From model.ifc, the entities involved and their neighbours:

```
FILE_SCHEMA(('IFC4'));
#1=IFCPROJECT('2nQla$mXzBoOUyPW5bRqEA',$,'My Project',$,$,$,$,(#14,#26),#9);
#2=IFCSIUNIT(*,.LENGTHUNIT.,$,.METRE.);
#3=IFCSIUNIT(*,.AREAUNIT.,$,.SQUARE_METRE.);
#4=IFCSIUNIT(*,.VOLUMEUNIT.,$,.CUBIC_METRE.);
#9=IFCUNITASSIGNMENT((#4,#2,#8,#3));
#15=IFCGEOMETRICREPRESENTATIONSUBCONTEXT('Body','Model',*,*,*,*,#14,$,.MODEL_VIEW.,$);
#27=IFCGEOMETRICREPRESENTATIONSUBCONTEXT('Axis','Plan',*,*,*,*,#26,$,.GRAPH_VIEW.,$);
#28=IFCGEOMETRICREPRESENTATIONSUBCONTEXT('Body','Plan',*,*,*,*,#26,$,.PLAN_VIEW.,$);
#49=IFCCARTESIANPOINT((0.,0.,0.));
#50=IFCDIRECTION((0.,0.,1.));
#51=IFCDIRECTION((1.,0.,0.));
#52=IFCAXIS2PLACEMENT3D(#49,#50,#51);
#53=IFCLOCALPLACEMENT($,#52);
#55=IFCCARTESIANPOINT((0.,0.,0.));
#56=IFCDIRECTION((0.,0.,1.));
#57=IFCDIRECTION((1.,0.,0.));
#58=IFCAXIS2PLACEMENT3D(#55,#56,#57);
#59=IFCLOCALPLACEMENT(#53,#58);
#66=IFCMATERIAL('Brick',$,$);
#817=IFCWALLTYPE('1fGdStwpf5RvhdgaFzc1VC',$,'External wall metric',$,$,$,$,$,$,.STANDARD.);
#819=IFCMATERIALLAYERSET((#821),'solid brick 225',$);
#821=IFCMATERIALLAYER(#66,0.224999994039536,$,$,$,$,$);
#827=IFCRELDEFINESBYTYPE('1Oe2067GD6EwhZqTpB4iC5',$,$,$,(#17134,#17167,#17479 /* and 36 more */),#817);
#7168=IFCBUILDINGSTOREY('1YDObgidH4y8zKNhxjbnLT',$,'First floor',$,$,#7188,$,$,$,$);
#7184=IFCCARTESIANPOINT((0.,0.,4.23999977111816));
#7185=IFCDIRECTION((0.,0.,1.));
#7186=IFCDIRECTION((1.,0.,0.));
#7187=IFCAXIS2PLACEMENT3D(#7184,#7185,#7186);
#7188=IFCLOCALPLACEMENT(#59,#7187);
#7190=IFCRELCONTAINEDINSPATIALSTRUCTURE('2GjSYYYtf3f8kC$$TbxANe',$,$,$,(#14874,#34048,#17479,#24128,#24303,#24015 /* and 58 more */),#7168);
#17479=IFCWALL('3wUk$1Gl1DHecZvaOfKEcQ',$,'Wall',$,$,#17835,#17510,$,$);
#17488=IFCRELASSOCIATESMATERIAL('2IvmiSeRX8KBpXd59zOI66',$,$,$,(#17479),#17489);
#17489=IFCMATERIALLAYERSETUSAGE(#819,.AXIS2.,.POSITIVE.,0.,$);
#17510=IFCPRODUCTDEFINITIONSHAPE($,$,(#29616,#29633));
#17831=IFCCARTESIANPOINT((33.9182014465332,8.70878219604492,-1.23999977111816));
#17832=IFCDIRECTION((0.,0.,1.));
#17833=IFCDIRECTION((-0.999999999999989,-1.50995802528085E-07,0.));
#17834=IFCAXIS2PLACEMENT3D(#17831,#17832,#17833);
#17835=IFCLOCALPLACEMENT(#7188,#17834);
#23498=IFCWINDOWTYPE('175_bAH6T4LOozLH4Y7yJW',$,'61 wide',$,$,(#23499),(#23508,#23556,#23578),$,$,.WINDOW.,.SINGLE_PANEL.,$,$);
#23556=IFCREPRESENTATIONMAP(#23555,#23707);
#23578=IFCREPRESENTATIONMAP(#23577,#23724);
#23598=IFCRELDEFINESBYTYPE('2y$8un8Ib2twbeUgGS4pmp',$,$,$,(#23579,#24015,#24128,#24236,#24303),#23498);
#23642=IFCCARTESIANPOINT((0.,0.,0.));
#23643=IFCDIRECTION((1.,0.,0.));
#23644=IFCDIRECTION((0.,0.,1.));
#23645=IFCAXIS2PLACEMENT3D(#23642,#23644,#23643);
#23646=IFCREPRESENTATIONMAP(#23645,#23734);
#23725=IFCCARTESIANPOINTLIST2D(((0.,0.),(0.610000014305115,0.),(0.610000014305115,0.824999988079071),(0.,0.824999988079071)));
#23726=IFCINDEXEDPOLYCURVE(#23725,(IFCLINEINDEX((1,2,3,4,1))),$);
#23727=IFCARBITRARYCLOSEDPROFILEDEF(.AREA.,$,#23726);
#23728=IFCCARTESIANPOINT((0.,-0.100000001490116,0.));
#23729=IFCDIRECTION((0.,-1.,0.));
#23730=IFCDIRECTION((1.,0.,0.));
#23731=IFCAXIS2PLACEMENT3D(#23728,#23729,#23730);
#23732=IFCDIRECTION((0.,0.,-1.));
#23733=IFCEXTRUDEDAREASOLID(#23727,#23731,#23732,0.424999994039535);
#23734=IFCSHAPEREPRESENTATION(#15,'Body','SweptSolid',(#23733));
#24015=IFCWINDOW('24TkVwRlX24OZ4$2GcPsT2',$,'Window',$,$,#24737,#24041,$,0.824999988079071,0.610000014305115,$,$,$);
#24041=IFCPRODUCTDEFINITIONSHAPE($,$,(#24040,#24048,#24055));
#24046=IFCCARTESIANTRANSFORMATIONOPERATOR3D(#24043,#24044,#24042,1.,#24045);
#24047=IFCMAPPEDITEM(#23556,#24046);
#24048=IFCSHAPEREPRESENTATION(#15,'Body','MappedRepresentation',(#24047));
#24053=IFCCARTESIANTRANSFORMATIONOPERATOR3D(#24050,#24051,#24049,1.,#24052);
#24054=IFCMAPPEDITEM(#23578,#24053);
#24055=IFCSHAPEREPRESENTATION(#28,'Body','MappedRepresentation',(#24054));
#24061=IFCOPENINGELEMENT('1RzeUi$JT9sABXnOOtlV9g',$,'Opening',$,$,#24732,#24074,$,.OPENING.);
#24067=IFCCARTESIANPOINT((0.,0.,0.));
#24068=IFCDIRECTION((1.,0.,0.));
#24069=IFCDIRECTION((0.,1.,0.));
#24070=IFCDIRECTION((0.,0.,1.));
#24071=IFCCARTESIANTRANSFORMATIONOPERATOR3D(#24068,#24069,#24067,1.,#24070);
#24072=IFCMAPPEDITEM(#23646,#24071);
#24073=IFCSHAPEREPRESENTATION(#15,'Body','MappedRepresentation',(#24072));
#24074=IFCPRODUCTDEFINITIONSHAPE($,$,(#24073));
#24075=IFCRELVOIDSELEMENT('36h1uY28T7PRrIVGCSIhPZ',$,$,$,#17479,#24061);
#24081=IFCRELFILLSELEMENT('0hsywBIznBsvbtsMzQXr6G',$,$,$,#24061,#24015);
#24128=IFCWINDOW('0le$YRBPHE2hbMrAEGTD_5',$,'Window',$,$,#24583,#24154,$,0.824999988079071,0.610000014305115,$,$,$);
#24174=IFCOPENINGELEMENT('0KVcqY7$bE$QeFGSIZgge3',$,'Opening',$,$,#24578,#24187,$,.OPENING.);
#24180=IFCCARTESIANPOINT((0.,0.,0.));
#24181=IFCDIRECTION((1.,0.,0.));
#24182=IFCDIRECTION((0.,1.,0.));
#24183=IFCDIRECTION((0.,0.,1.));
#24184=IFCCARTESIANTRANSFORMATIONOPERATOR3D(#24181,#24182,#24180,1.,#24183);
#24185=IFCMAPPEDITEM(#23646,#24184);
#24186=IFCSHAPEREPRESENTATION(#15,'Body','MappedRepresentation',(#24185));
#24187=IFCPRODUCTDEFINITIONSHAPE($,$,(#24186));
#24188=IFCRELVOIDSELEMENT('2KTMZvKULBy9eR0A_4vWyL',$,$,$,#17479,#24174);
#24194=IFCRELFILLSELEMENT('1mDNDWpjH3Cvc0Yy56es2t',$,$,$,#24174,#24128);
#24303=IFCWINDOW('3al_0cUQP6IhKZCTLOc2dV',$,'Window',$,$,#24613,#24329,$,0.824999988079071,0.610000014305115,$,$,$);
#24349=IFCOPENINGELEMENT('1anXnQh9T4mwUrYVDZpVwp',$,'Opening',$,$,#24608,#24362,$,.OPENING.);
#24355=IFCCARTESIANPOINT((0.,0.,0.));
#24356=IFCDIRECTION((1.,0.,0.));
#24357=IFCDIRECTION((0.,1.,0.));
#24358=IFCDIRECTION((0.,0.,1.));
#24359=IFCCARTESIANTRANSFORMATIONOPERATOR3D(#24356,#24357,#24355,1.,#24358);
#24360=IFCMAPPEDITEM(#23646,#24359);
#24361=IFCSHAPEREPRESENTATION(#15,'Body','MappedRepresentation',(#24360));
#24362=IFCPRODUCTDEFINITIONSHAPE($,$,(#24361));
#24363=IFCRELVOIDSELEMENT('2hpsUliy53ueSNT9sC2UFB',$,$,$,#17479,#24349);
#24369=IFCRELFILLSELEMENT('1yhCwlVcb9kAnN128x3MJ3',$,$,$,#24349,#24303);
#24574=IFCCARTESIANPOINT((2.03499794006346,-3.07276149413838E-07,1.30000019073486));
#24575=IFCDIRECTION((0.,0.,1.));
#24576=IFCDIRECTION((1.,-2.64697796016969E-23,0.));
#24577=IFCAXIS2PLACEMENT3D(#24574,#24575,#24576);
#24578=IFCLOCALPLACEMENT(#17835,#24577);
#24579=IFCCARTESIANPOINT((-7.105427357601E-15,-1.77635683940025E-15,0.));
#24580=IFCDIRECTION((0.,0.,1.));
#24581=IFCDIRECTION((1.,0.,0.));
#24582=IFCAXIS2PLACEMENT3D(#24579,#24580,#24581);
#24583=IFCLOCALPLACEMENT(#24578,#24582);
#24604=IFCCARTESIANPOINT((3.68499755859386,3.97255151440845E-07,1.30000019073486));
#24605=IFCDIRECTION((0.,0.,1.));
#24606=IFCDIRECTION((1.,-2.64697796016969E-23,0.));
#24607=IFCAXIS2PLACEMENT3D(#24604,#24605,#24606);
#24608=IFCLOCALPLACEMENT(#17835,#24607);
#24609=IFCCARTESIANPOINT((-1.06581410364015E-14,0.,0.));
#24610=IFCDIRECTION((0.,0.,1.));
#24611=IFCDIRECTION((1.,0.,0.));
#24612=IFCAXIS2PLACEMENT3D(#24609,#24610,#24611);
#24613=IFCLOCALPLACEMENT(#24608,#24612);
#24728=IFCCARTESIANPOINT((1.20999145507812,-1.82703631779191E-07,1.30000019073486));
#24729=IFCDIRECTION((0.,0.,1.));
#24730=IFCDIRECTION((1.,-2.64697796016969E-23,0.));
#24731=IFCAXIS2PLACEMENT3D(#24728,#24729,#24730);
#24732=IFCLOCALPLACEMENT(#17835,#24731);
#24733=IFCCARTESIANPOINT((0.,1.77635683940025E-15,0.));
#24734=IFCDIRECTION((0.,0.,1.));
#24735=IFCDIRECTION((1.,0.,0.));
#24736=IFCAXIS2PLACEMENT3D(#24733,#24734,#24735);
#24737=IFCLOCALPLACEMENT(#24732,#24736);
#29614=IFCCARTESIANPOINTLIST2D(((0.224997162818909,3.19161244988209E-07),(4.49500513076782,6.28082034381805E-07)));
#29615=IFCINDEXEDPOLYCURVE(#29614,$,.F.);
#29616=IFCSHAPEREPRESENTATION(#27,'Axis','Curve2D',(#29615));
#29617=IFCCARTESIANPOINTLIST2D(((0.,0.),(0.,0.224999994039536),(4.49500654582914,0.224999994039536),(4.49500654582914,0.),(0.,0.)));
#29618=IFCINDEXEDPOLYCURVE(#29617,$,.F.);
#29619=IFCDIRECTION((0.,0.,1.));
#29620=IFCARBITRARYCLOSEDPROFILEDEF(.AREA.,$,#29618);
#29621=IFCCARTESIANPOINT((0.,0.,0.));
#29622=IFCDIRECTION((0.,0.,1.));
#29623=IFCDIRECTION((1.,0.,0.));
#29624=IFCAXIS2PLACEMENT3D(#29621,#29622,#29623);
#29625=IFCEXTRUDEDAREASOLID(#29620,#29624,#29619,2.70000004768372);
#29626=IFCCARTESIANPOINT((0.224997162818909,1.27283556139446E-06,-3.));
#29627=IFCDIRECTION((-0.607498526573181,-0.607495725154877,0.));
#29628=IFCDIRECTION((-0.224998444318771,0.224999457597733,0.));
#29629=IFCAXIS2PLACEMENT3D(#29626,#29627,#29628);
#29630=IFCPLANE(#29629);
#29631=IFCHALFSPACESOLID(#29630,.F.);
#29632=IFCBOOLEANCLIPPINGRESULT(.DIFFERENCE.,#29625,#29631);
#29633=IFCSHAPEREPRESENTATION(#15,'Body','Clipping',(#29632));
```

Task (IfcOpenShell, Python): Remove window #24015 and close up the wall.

```python
import ifcopenshell
import ifcopenshell.api.feature
import ifcopenshell.api.root
import ifcopenshell.geom
import ifcopenshell.util.shape

model = ifcopenshell.open("model.ifc")
settings = ifcopenshell.geom.settings()


def volume(element):
    """Net volume in cubic metres, openings subtracted."""
    shape = ifcopenshell.geom.create_shape(settings, element)
    return ifcopenshell.util.shape.get_volume(shape.geometry)


window = model.by_id(24015)
opening = window.FillsVoids[0].RelatingOpeningElement
wall = opening.VoidsElements[0].RelatingBuildingElement
before = volume(wall)

ifcopenshell.api.root.remove_product(model, product=window)
ifcopenshell.api.feature.remove_feature(model, feature=opening)

after = volume(wall)

print(f"wall volume {before:.3f} -> {after:.3f} m3")

model.write("model-out.ifc")
```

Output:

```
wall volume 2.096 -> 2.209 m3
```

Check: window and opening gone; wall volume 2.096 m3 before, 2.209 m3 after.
